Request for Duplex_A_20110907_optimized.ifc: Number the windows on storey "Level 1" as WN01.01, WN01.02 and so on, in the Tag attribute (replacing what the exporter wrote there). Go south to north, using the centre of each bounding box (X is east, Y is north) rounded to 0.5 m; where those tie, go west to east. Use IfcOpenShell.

First a look at what the model holds.

```python
import ifcopenshell
import ifcopenshell.util.element
import ifcopenshell.util.placement

model = ifcopenshell.open("Duplex_A_20110907_optimized.ifc")
print(model.schema)
storey = next(s for s in model.by_type("IfcBuildingStorey") if s.Name == "Level 1")
windows = [e for e in ifcopenshell.util.element.get_decomposition(storey) if e.is_a("IfcWindow")]
for e in sorted(windows, key=lambda e: e.id()):
    origin = ifcopenshell.util.placement.get_local_placement(e.ObjectPlacement)[:3, 3]
    print(e.id(), e.Tag, e.Name, origin.round(2) + 0.0, sep=" | ")
```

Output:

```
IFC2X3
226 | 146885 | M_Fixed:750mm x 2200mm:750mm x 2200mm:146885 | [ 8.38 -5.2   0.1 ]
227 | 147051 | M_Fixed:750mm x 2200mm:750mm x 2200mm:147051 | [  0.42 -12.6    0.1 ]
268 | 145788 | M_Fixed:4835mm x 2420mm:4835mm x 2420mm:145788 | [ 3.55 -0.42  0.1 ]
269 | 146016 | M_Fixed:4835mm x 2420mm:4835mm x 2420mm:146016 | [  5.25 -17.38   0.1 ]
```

```python
import ifcopenshell
import ifcopenshell.geom
import ifcopenshell.util.element
import ifcopenshell.util.shape

model = ifcopenshell.open("Duplex_A_20110907_optimized.ifc")
settings = ifcopenshell.geom.settings()
settings.set("use-world-coords", True)


def centre(element):
    shape = ifcopenshell.geom.create_shape(settings, element)
    return ifcopenshell.util.shape.get_bbox_centroid(shape.geometry)


storey = next(s for s in model.by_type("IfcBuildingStorey") if s.Name == "Level 1")
windows = [e for e in ifcopenshell.util.element.get_decomposition(storey) if e.is_a("IfcWindow")]

# Insertion points can sit at a corner or the storey origin, so sort by the geometry (in metres).
centres = {e: centre(e) for e in windows}
windows.sort(key=lambda e: (round(centres[e][1] / 0.5), centres[e][0]))

for i, e in enumerate(windows, start=1):
    number = f"WN01.{i:02d}"
    e.Tag = number
    print(e.id(), number)

model.write("Duplex_A_20110907_optimized_v2.ifc")
```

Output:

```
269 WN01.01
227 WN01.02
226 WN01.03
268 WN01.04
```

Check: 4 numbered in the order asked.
